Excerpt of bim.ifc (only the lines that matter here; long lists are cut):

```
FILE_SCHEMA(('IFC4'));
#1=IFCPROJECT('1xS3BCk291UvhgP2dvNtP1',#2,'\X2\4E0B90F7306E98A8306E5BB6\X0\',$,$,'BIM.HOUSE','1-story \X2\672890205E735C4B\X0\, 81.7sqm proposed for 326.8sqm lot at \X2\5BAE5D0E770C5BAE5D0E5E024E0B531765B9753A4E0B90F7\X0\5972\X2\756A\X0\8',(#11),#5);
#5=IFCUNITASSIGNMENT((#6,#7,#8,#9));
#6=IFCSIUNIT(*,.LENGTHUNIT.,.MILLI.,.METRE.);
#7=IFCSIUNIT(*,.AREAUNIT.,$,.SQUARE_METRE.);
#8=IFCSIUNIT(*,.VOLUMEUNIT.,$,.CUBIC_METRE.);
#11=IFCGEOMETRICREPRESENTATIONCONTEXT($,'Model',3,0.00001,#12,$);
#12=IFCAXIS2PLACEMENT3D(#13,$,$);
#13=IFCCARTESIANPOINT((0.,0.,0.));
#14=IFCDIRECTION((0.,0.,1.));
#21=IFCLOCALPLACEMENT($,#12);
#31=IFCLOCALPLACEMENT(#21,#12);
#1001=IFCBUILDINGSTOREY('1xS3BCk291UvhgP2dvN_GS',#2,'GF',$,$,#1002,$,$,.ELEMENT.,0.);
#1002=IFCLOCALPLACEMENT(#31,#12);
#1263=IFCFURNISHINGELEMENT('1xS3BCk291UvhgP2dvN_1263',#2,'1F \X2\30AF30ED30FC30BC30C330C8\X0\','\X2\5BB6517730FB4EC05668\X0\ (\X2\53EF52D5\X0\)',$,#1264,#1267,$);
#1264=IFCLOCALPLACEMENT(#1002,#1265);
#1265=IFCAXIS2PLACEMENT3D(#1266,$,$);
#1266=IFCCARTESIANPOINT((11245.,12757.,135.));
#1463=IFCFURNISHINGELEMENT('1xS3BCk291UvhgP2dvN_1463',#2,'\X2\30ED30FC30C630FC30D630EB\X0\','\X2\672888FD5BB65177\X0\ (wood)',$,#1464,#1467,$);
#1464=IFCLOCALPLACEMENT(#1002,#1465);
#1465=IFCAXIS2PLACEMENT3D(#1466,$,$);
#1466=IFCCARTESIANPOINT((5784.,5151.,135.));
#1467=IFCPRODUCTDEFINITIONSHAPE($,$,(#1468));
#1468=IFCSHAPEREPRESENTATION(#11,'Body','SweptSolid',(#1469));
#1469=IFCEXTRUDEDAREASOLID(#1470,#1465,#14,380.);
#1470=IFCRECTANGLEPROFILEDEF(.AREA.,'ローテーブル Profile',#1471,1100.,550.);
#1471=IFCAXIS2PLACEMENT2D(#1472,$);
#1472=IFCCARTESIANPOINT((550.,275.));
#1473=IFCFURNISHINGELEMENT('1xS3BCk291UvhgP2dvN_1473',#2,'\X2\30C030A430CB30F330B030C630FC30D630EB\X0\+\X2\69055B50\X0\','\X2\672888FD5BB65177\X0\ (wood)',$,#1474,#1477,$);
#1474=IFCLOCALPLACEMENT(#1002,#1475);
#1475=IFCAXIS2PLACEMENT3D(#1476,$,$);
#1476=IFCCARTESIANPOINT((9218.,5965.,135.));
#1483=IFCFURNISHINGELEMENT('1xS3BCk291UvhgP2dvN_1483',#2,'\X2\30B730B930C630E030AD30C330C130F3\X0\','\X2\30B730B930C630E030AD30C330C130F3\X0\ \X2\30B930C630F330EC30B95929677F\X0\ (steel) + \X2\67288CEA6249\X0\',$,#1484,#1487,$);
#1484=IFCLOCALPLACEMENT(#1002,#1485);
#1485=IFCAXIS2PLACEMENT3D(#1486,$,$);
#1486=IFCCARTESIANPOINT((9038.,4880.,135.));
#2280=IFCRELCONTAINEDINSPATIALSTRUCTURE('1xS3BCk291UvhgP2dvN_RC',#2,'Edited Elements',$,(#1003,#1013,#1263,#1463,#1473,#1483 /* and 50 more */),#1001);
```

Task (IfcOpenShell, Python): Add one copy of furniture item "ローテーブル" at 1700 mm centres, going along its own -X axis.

```python
import ifcopenshell
import ifcopenshell.api.geometry
import ifcopenshell.api.root
import ifcopenshell.util.element
import ifcopenshell.util.placement
import ifcopenshell.util.unit

model = ifcopenshell.open("bim.ifc")
unit_scale = ifcopenshell.util.unit.calculate_unit_scale(model)


def reuse_history(source, copy):
    """copy_class also copies each property set's owner history, people and application; keep the originals."""
    for rel in copy.IsDefinedBy:
        if rel.is_a("IfcRelDefinesByProperties") and (history := rel.RelatingPropertyDefinition.OwnerHistory):
            rel.RelatingPropertyDefinition.OwnerHistory = source.OwnerHistory
            ifcopenshell.util.element.remove_deep2(model, history)


source = model.by_guid("1xS3BCk291UvhgP2dvN_1463")
base = ifcopenshell.util.placement.get_local_placement(source.ObjectPlacement)
step = -base[:3, 0] * 1.7 / unit_scale

for i in range(1, 2):
    copy = ifcopenshell.api.root.copy_class(model, product=source)
    copy.Representation = ifcopenshell.util.element.copy_deep(
        model, source.Representation, exclude=["IfcGeometricRepresentationContext", "IfcRepresentationMap"]
    )
    reuse_history(source, copy)
    matrix = base.copy()
    matrix[:3, 3] += i * step
    print("added at", matrix[:3, 3].round(3) + 0.0)
    ifcopenshell.api.geometry.edit_object_placement(model, product=copy, matrix=matrix, is_si=False)

model.write("bim_edited.ifc")
```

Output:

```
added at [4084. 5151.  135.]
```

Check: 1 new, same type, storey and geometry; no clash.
